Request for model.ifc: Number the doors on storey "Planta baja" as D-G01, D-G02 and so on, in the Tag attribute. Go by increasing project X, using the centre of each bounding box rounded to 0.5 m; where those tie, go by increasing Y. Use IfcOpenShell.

First a look at what the model holds.

```python
import ifcopenshell
import ifcopenshell.util.element
import ifcopenshell.util.placement

model = ifcopenshell.open("model.ifc")
print(model.schema)
storey = next(s for s in model.by_type("IfcBuildingStorey") if s.Name == "Planta baja")
doors = [e for e in ifcopenshell.util.element.get_decomposition(storey) if e.is_a("IfcDoor")]
for e in sorted(doors, key=lambda e: e.id()):
    origin = ifcopenshell.util.placement.get_local_placement(e.ObjectPlacement)[:3, 3]
    print(e.id(), e.Tag, e.Name, origin.round(2) + 0.0, sep=" | ")
```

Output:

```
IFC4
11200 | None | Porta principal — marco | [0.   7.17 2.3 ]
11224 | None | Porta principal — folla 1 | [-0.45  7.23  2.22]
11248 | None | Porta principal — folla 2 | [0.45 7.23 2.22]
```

```python
import ifcopenshell
import ifcopenshell.geom
import ifcopenshell.util.element
import ifcopenshell.util.shape

model = ifcopenshell.open("model.ifc")
settings = ifcopenshell.geom.settings()
settings.set("use-world-coords", True)


def centre(element):
    shape = ifcopenshell.geom.create_shape(settings, element)
    return ifcopenshell.util.shape.get_bbox_centroid(shape.geometry)


storey = next(s for s in model.by_type("IfcBuildingStorey") if s.Name == "Planta baja")
doors = [e for e in ifcopenshell.util.element.get_decomposition(storey) if e.is_a("IfcDoor")]

# Insertion points can sit at a corner or the storey origin, so sort by the geometry (in metres).
centres = {e: centre(e) for e in doors}
doors.sort(key=lambda e: (round(centres[e][0] / 0.5), centres[e][1]))

for i, e in enumerate(doors, start=1):
    number = f"D-G{i:02d}"
    e.Tag = number
    print(e.id(), number)

model.write("model_rev.ifc")
```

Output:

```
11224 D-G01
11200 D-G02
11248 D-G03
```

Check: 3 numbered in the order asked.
